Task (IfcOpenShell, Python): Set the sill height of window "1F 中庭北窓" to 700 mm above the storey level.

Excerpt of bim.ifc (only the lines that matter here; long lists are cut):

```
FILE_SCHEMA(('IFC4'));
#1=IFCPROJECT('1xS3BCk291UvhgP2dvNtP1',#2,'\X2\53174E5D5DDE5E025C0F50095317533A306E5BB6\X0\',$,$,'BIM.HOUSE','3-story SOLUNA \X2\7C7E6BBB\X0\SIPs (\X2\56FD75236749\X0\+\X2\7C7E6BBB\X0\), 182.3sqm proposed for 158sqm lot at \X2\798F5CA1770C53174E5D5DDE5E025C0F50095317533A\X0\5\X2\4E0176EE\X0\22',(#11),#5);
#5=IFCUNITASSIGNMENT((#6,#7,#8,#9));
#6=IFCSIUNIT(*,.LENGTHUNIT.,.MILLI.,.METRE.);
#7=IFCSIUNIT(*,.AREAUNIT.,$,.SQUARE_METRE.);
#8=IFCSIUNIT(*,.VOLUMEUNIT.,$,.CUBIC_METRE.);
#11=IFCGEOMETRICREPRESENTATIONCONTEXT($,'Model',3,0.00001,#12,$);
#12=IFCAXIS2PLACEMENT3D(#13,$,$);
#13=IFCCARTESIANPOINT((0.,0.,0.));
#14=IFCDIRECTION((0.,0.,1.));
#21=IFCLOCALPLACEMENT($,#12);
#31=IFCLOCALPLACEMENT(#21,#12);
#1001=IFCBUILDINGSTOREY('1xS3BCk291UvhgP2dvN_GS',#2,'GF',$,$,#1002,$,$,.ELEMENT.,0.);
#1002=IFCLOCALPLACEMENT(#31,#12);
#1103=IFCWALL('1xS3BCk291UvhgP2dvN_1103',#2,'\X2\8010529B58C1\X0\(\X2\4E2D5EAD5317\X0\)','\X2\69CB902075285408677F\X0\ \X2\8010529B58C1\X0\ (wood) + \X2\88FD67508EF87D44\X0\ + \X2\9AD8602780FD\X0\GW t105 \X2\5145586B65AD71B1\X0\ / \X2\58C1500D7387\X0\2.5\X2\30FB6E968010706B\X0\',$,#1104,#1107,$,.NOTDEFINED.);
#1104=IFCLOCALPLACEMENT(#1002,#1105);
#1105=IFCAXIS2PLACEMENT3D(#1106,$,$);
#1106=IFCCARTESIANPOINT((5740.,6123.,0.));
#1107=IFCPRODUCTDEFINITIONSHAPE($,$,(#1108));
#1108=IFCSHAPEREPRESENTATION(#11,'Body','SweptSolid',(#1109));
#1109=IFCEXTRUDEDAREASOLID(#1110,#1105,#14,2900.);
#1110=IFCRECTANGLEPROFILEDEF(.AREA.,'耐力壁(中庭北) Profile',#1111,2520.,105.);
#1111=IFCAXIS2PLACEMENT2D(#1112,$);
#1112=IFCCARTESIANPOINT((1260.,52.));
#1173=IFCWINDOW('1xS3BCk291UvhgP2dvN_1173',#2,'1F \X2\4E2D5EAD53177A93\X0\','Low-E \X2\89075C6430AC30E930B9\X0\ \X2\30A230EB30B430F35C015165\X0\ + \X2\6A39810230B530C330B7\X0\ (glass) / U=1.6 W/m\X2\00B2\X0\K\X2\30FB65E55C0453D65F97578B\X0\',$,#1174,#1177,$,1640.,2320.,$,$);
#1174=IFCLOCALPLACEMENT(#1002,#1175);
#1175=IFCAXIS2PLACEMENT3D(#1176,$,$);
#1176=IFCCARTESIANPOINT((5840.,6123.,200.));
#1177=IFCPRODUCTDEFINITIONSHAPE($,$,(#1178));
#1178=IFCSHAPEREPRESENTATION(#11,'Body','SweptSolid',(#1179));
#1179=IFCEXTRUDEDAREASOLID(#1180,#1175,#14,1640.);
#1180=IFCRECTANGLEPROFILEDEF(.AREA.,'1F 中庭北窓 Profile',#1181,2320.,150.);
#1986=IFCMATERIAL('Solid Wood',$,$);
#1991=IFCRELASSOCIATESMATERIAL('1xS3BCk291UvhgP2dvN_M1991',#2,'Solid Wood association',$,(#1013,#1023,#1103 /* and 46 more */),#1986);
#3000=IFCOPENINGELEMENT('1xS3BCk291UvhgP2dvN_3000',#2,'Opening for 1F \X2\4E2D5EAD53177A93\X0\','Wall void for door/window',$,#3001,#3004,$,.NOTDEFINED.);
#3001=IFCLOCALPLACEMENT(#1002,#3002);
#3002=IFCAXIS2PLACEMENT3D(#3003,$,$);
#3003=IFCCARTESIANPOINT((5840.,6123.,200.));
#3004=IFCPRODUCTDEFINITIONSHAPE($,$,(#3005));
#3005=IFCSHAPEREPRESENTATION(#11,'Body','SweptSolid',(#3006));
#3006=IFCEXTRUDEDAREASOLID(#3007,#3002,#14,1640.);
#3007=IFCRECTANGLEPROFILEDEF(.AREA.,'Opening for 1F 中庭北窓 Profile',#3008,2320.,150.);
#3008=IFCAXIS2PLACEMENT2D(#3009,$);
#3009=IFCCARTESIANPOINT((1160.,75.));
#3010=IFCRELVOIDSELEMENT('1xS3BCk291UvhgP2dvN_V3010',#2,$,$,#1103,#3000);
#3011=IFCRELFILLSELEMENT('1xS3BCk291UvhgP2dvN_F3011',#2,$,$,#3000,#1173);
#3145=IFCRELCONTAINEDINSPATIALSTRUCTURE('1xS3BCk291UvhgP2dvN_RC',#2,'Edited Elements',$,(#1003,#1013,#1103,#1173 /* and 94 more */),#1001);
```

```python
import numpy as np
import ifcopenshell
import ifcopenshell.api.geometry
import ifcopenshell.geom
import ifcopenshell.util.element
import ifcopenshell.util.placement
import ifcopenshell.util.shape
import ifcopenshell.util.unit

model = ifcopenshell.open("bim.ifc")
unit_scale = ifcopenshell.util.unit.calculate_unit_scale(model)

window = model.by_guid("1xS3BCk291UvhgP2dvN_1173")
opening = window.FillsVoids[0].RelatingOpeningElement
storey = ifcopenshell.util.element.get_container(window, ifc_class="IfcBuildingStorey")
level = ifcopenshell.util.placement.get_local_placement(storey.ObjectPlacement)[2, 3]

# The opening's origin need not be at the sill, so measure its lowest point.
shape = ifcopenshell.geom.create_shape(ifcopenshell.geom.settings(), opening)
bottom = ifcopenshell.util.shape.get_shape_bottom_elevation(shape, shape.geometry) / unit_scale
dz = level + 0.7 / unit_scale - bottom

shift = np.array([0.0, 0.0, dz])
# The window is not placed relative to its opening, so move both.
for product in (opening, window):
    matrix = ifcopenshell.util.placement.get_local_placement(product.ObjectPlacement)
    matrix[:3, 3] += shift
    ifcopenshell.api.geometry.edit_object_placement(model, product=product, matrix=matrix, is_si=False)

print(f"moved by {dz * unit_scale:+.3f} m")

model.write("bim-out.ifc")
```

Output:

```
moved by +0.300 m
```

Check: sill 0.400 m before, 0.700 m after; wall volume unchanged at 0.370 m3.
